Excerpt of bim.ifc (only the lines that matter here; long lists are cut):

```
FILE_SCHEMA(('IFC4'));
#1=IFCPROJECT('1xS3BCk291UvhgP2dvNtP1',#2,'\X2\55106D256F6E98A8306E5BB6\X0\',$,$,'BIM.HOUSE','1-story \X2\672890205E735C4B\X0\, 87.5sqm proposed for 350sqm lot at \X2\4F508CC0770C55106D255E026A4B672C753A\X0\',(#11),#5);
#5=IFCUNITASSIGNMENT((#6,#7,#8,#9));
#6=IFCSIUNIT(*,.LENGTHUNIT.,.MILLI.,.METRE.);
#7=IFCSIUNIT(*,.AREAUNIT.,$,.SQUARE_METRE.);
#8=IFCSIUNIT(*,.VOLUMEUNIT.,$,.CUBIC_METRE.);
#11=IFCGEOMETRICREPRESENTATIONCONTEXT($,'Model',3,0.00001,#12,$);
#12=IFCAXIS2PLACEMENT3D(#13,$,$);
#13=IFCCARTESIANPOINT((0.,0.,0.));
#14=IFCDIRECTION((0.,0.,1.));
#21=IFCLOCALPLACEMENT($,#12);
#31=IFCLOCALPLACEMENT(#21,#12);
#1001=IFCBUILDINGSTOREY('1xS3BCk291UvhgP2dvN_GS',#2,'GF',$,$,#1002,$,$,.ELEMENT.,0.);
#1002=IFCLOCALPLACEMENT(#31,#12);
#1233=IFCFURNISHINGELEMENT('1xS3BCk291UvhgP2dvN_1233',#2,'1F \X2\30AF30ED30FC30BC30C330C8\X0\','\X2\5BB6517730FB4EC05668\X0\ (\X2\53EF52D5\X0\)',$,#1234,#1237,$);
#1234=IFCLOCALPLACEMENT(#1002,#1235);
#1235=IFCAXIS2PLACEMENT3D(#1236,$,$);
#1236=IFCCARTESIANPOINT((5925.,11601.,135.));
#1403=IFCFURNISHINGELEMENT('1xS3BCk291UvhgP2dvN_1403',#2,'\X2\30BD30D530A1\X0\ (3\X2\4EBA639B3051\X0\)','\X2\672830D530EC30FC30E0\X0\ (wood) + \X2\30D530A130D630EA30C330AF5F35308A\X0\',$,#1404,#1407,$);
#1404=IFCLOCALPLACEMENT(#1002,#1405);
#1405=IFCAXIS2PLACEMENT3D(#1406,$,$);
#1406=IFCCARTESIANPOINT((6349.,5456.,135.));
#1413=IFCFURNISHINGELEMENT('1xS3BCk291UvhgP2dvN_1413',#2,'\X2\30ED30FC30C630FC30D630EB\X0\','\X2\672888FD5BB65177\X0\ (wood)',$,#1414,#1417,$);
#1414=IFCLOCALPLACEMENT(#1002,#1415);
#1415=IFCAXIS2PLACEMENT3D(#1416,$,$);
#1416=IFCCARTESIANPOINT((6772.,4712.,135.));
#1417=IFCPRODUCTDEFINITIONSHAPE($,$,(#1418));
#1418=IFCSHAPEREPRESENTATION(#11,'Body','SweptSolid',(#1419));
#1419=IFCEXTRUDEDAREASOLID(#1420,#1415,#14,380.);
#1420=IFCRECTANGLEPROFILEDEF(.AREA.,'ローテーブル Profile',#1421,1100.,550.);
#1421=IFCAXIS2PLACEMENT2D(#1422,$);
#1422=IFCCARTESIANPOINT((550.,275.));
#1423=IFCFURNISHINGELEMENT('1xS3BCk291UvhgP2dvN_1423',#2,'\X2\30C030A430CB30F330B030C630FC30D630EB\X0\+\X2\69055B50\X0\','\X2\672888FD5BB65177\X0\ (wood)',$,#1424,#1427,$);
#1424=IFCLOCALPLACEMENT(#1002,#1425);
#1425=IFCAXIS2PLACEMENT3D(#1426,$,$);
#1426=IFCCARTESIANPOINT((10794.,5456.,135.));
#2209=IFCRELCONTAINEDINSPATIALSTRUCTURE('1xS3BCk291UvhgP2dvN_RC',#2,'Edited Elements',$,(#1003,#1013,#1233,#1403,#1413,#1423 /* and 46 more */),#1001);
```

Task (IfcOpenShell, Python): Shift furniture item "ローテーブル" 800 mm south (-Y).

```python
import ifcopenshell
import ifcopenshell.api.geometry
import ifcopenshell.util.placement

model = ifcopenshell.open("bim.ifc")

item = model.by_id(1413)
matrix = ifcopenshell.util.placement.get_local_placement(item.ObjectPlacement)
matrix[1, 3] -= 800.0
ifcopenshell.api.geometry.edit_object_placement(model, product=item, matrix=matrix, is_si=False)

print(ifcopenshell.util.placement.get_local_placement(item.ObjectPlacement).round(3) + 0.0)

model.write("bim-out.ifc")
```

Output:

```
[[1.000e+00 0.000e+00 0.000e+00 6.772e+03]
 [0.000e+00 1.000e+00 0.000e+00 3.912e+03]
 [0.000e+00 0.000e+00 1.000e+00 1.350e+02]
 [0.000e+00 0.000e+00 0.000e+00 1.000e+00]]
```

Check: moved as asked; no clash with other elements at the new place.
